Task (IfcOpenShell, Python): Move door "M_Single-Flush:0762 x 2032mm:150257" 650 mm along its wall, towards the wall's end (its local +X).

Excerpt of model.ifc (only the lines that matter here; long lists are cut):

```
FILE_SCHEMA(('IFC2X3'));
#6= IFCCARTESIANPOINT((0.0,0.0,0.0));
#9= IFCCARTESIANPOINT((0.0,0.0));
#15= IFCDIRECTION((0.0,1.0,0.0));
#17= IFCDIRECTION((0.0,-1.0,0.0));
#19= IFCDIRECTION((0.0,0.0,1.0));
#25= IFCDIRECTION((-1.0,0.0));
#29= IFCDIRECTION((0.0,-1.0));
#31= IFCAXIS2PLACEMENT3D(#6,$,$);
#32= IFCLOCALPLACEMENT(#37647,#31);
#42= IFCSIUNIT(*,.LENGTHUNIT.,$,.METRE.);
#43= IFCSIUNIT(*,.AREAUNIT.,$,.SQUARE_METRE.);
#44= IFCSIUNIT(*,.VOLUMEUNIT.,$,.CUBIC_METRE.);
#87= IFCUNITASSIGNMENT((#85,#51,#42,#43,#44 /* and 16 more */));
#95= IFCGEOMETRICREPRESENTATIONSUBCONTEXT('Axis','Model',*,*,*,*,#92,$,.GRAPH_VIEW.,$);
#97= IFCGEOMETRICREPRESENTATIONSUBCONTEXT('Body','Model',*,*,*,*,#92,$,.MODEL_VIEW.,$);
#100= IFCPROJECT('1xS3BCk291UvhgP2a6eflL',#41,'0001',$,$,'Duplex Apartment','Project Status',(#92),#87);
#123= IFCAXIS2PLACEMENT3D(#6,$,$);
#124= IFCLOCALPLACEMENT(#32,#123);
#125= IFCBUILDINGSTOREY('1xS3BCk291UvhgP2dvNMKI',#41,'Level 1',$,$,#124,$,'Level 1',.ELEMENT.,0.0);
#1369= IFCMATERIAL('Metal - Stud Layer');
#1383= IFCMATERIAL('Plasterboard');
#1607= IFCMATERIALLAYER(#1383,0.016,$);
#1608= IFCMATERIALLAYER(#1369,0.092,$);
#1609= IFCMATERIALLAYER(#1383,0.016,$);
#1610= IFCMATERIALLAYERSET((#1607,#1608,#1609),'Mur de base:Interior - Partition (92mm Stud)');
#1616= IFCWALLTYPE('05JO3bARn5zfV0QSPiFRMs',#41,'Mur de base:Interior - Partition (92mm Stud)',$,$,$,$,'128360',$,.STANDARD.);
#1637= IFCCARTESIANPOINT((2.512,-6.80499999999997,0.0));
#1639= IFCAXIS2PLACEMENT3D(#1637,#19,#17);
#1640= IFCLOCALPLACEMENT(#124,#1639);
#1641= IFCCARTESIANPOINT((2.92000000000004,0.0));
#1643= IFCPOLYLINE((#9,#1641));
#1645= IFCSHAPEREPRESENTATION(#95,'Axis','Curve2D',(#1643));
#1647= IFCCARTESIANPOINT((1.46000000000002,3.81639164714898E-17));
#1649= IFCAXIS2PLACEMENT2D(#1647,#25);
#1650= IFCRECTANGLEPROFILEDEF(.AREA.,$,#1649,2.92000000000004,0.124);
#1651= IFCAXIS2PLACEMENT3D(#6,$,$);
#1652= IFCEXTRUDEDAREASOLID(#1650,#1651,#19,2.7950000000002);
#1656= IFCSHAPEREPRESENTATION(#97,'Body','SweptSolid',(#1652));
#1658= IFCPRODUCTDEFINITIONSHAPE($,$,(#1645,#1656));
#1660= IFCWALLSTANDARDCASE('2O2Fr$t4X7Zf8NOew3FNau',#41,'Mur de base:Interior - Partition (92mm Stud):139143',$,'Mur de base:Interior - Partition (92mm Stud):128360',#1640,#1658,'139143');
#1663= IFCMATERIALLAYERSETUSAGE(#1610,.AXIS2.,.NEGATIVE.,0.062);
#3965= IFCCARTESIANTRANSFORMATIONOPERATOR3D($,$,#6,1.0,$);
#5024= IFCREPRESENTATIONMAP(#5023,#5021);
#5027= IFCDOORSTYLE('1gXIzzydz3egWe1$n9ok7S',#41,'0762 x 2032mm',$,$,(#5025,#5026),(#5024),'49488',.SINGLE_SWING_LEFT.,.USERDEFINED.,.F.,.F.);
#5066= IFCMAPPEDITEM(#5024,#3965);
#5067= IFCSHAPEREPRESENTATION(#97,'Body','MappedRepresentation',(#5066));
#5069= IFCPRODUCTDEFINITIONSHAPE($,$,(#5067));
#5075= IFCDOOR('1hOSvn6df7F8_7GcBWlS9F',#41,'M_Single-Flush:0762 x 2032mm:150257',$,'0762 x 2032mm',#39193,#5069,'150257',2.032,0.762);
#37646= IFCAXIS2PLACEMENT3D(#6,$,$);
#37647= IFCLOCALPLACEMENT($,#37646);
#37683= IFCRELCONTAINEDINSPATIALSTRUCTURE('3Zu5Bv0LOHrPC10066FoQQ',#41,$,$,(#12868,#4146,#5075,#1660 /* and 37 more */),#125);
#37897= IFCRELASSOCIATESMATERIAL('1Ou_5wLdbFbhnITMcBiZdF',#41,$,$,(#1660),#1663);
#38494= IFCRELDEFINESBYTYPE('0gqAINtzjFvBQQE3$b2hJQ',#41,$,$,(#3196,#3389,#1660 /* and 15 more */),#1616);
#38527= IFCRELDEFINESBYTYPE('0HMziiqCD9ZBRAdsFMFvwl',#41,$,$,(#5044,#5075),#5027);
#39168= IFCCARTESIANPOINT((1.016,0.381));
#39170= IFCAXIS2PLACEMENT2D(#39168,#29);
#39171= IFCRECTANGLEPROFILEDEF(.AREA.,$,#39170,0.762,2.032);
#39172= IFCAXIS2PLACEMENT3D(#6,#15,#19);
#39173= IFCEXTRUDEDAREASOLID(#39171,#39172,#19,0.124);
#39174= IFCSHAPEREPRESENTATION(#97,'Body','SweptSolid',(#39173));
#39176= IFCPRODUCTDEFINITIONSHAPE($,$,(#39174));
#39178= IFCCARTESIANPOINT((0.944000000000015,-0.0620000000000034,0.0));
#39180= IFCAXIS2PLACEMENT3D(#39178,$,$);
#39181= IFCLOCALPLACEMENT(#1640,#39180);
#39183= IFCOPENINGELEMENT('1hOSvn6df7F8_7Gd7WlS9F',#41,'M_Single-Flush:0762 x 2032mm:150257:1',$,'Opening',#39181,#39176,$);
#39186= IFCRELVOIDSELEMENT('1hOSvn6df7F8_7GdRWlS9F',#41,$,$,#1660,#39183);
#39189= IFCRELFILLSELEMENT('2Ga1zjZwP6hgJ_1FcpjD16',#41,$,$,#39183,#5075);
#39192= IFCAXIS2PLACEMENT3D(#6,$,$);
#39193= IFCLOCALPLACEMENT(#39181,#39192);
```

```python
import ifcopenshell
import ifcopenshell.api.geometry
import ifcopenshell.util.placement
import ifcopenshell.util.unit

model = ifcopenshell.open("model.ifc")
unit_scale = ifcopenshell.util.unit.calculate_unit_scale(model)

door = model.by_id(5075)
opening = door.FillsVoids[0].RelatingOpeningElement
wall = opening.VoidsElements[0].RelatingBuildingElement

wall_matrix = ifcopenshell.util.placement.get_local_placement(wall.ObjectPlacement)
shift = wall_matrix[:3, 0] * 0.65 / unit_scale
before = ifcopenshell.util.placement.get_local_placement(door.ObjectPlacement)[:3, 3].copy()

# The door is placed relative to its opening, so it follows when the opening moves.
matrix = ifcopenshell.util.placement.get_local_placement(opening.ObjectPlacement)
matrix[:3, 3] += shift
ifcopenshell.api.geometry.edit_object_placement(
    model, product=opening, matrix=matrix, is_si=False, should_transform_children=True
)

after = ifcopenshell.util.placement.get_local_placement(door.ObjectPlacement)[:3, 3]
print("door moved by", (after - before).round(3) + 0.0)

model.write("model_rev.ifc")
```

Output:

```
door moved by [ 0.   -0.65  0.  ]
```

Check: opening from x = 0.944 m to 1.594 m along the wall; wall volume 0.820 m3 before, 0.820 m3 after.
